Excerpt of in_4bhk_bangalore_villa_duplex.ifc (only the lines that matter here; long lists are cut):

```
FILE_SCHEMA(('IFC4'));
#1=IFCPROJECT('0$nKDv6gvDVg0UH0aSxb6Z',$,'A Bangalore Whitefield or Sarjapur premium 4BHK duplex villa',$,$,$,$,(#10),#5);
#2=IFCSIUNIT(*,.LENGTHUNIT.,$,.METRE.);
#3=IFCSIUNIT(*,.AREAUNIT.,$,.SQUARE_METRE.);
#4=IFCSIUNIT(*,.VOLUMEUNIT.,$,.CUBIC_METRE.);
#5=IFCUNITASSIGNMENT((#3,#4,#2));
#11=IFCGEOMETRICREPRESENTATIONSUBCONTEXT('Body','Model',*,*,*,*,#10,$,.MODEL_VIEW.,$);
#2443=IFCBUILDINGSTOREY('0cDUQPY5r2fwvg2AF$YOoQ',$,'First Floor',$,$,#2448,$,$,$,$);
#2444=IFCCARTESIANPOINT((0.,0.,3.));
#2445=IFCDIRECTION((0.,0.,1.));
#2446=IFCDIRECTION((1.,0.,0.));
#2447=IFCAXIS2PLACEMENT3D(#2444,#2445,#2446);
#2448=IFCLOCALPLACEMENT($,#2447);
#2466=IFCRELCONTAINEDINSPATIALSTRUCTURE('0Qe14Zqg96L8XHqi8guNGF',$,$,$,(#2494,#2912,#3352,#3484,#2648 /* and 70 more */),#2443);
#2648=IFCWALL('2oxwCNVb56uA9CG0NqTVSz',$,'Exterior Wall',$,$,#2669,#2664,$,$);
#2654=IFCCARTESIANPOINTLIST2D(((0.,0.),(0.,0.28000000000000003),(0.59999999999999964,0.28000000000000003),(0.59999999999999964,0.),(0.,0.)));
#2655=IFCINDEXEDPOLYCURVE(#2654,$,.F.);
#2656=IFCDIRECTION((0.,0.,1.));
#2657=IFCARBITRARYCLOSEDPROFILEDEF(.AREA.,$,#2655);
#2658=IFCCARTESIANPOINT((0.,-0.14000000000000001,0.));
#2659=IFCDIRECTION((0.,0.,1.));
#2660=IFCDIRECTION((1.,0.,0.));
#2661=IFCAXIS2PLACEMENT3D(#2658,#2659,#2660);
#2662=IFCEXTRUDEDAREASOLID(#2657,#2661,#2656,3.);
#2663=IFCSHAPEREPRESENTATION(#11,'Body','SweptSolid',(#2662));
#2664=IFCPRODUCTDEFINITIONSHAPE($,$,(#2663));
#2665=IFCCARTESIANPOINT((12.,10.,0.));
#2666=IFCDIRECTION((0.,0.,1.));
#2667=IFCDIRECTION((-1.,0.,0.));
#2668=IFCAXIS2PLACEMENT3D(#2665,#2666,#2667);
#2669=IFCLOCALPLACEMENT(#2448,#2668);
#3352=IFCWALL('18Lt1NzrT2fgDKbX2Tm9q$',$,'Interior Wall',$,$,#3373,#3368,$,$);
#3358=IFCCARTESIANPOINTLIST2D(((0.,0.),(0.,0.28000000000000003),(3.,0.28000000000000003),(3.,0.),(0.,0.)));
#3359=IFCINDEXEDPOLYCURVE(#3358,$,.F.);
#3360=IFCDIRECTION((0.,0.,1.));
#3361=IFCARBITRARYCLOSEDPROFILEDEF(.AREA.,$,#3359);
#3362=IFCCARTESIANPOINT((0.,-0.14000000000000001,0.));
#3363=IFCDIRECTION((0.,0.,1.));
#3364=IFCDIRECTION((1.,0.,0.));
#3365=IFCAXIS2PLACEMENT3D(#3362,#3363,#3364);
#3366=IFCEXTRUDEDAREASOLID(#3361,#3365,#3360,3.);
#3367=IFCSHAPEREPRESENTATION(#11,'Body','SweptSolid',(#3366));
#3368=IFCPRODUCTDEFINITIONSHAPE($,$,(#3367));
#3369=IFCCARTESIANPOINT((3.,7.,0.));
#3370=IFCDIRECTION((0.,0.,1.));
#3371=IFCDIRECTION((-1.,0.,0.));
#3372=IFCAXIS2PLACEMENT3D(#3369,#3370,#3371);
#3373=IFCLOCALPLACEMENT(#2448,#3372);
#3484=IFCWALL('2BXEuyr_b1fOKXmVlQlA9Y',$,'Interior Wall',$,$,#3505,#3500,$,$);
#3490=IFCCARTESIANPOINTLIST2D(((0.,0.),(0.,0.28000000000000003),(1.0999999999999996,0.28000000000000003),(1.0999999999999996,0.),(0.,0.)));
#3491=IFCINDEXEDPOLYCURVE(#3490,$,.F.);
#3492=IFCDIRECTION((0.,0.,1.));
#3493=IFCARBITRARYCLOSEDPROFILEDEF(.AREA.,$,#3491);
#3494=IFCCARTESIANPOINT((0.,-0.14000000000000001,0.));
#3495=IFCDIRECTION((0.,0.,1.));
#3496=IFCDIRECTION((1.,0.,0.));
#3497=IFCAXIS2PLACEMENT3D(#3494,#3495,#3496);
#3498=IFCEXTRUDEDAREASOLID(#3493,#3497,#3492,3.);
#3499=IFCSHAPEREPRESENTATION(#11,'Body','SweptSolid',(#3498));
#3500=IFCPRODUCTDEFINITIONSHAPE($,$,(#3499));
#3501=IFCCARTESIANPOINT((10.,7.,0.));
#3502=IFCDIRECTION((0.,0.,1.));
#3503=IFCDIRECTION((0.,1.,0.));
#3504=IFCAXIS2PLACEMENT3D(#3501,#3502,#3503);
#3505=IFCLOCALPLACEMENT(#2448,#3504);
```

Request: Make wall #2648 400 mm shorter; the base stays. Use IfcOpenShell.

```python
import ifcopenshell
import ifcopenshell.geom
import ifcopenshell.util.representation
import ifcopenshell.util.shape

model = ifcopenshell.open("in_4bhk_bangalore_villa_duplex.ifc")
settings = ifcopenshell.geom.settings()


def volume(element):
    """Net volume in cubic metres, openings subtracted."""
    shape = ifcopenshell.geom.create_shape(settings, element)
    return ifcopenshell.util.shape.get_volume(shape.geometry)


wall = model.by_guid("2oxwCNVb56uA9CG0NqTVSz")
before = volume(wall)

body = ifcopenshell.util.representation.get_representation(wall, "Model", "Body")
solid = body.Items[0]
old_height = solid.Depth
solid.Depth -= 0.4
after = volume(wall)

print(f"height {old_height:g} -> {solid.Depth:g}, volume {before:.3f} -> {after:.3f} m3")

model.write("in_4bhk_bangalore_villa_duplex_rev.ifc")
```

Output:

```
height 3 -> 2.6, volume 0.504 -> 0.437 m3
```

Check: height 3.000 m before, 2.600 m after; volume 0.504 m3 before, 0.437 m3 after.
